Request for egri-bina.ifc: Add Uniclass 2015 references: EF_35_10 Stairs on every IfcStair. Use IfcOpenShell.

First a look at what the model holds.

```python
import ifcopenshell

model = ifcopenshell.open("egri-bina.ifc")
print(model.schema)
print("classifications:", [c.Name for c in model.by_type("IfcClassification")])
for ifc_class in ("IfcDoor", "IfcRoof", "IfcStair", "IfcWall", "IfcWindow"):
    print(ifc_class, len(model.by_type(ifc_class)))
```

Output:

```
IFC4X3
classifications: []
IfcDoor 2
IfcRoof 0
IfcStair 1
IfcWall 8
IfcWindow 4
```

```python
import ifcopenshell
import ifcopenshell.api.classification

model = ifcopenshell.open("egri-bina.ifc")

system = ifcopenshell.api.classification.add_classification(model, classification="Uniclass 2015")

codes = {
    "IfcStair": ("EF_35_10", "Stairs"),
}
for ifc_class, (code, name) in codes.items():
    products = model.by_type(ifc_class)
    ifcopenshell.api.classification.add_reference(
        model, products=products, classification=system, identification=code, name=name
    )
    print(code, len(products))

model.write("egri-bina_edited.ifc")
```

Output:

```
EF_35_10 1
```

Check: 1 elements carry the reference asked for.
